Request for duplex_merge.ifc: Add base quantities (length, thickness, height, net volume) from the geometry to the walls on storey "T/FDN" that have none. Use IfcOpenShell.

First a look at what the model holds.

```python
import ifcopenshell
import ifcopenshell.util.element
import ifcopenshell.util.unit

model = ifcopenshell.open("duplex_merge.ifc")
print(model.schema)
for unit_type in ("LENGTHUNIT", "AREAUNIT", "VOLUMEUNIT"):
    print(unit_type, ifcopenshell.util.unit.calculate_unit_scale(model, unit_type))
storey = next(s for s in model.by_type("IfcBuildingStorey") if s.Name == "T/FDN")
walls = [e for e in ifcopenshell.util.element.get_decomposition(storey) if e.is_a("IfcWall")]
for e in sorted(walls, key=lambda e: e.id()):
    print(e.id(), e.is_a(), e.Name, list(ifcopenshell.util.element.get_psets(e, qtos_only=True)), sep=" | ")
```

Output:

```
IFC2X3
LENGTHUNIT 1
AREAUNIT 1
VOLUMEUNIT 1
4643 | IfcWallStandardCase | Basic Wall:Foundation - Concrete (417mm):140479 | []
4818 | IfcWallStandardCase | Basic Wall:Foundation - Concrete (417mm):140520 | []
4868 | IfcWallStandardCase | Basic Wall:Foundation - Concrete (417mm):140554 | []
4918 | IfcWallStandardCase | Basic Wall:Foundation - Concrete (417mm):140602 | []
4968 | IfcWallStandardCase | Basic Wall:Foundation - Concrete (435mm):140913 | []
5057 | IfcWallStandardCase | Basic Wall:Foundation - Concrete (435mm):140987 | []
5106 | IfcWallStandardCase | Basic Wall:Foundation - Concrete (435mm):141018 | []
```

```python
import ifcopenshell
import ifcopenshell.api.pset
import ifcopenshell.geom
import ifcopenshell.util.element
import ifcopenshell.util.shape
import ifcopenshell.util.unit

model = ifcopenshell.open("duplex_merge.ifc")
unit_scale = ifcopenshell.util.unit.calculate_unit_scale(model)
volume_scale = ifcopenshell.util.unit.calculate_unit_scale(model, "VOLUMEUNIT")
settings = ifcopenshell.geom.settings()

storey = next(s for s in model.by_type("IfcBuildingStorey") if s.Name == "T/FDN")
walls = [e for e in ifcopenshell.util.element.get_decomposition(storey) if e.is_a("IfcWall")]

for e in sorted(walls, key=lambda e: e.id()):
    if ifcopenshell.util.element.get_psets(e, qtos_only=True, should_inherit=False):
        continue
    # Geometry comes back in metres, in the element's own axes.
    shape = ifcopenshell.geom.create_shape(settings, e)
    values = {
        "Length": ifcopenshell.util.shape.get_x(shape.geometry) / unit_scale,
        "Width": ifcopenshell.util.shape.get_y(shape.geometry) / unit_scale,
        "Height": ifcopenshell.util.shape.get_z(shape.geometry) / unit_scale,
        "NetVolume": ifcopenshell.util.shape.get_volume(shape.geometry) / volume_scale,
    }
    qto = ifcopenshell.api.pset.add_qto(model, product=e, name="BaseQuantities")
    ifcopenshell.api.pset.edit_qto(model, qto=qto, properties=values)
    print(e.id(), {k: round(v, 3) for k, v in values.items()})

model.write("duplex_merge_v2.ifc")
```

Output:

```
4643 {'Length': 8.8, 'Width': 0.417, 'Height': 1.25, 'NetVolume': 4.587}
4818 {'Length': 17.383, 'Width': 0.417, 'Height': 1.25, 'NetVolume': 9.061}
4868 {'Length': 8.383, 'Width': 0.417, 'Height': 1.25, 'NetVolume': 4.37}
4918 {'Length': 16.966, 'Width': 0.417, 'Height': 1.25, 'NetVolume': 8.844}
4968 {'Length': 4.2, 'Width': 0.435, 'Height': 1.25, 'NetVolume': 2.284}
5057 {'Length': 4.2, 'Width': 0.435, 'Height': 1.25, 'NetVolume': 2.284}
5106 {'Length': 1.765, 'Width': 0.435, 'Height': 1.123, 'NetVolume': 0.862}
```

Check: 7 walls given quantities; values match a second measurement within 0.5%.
